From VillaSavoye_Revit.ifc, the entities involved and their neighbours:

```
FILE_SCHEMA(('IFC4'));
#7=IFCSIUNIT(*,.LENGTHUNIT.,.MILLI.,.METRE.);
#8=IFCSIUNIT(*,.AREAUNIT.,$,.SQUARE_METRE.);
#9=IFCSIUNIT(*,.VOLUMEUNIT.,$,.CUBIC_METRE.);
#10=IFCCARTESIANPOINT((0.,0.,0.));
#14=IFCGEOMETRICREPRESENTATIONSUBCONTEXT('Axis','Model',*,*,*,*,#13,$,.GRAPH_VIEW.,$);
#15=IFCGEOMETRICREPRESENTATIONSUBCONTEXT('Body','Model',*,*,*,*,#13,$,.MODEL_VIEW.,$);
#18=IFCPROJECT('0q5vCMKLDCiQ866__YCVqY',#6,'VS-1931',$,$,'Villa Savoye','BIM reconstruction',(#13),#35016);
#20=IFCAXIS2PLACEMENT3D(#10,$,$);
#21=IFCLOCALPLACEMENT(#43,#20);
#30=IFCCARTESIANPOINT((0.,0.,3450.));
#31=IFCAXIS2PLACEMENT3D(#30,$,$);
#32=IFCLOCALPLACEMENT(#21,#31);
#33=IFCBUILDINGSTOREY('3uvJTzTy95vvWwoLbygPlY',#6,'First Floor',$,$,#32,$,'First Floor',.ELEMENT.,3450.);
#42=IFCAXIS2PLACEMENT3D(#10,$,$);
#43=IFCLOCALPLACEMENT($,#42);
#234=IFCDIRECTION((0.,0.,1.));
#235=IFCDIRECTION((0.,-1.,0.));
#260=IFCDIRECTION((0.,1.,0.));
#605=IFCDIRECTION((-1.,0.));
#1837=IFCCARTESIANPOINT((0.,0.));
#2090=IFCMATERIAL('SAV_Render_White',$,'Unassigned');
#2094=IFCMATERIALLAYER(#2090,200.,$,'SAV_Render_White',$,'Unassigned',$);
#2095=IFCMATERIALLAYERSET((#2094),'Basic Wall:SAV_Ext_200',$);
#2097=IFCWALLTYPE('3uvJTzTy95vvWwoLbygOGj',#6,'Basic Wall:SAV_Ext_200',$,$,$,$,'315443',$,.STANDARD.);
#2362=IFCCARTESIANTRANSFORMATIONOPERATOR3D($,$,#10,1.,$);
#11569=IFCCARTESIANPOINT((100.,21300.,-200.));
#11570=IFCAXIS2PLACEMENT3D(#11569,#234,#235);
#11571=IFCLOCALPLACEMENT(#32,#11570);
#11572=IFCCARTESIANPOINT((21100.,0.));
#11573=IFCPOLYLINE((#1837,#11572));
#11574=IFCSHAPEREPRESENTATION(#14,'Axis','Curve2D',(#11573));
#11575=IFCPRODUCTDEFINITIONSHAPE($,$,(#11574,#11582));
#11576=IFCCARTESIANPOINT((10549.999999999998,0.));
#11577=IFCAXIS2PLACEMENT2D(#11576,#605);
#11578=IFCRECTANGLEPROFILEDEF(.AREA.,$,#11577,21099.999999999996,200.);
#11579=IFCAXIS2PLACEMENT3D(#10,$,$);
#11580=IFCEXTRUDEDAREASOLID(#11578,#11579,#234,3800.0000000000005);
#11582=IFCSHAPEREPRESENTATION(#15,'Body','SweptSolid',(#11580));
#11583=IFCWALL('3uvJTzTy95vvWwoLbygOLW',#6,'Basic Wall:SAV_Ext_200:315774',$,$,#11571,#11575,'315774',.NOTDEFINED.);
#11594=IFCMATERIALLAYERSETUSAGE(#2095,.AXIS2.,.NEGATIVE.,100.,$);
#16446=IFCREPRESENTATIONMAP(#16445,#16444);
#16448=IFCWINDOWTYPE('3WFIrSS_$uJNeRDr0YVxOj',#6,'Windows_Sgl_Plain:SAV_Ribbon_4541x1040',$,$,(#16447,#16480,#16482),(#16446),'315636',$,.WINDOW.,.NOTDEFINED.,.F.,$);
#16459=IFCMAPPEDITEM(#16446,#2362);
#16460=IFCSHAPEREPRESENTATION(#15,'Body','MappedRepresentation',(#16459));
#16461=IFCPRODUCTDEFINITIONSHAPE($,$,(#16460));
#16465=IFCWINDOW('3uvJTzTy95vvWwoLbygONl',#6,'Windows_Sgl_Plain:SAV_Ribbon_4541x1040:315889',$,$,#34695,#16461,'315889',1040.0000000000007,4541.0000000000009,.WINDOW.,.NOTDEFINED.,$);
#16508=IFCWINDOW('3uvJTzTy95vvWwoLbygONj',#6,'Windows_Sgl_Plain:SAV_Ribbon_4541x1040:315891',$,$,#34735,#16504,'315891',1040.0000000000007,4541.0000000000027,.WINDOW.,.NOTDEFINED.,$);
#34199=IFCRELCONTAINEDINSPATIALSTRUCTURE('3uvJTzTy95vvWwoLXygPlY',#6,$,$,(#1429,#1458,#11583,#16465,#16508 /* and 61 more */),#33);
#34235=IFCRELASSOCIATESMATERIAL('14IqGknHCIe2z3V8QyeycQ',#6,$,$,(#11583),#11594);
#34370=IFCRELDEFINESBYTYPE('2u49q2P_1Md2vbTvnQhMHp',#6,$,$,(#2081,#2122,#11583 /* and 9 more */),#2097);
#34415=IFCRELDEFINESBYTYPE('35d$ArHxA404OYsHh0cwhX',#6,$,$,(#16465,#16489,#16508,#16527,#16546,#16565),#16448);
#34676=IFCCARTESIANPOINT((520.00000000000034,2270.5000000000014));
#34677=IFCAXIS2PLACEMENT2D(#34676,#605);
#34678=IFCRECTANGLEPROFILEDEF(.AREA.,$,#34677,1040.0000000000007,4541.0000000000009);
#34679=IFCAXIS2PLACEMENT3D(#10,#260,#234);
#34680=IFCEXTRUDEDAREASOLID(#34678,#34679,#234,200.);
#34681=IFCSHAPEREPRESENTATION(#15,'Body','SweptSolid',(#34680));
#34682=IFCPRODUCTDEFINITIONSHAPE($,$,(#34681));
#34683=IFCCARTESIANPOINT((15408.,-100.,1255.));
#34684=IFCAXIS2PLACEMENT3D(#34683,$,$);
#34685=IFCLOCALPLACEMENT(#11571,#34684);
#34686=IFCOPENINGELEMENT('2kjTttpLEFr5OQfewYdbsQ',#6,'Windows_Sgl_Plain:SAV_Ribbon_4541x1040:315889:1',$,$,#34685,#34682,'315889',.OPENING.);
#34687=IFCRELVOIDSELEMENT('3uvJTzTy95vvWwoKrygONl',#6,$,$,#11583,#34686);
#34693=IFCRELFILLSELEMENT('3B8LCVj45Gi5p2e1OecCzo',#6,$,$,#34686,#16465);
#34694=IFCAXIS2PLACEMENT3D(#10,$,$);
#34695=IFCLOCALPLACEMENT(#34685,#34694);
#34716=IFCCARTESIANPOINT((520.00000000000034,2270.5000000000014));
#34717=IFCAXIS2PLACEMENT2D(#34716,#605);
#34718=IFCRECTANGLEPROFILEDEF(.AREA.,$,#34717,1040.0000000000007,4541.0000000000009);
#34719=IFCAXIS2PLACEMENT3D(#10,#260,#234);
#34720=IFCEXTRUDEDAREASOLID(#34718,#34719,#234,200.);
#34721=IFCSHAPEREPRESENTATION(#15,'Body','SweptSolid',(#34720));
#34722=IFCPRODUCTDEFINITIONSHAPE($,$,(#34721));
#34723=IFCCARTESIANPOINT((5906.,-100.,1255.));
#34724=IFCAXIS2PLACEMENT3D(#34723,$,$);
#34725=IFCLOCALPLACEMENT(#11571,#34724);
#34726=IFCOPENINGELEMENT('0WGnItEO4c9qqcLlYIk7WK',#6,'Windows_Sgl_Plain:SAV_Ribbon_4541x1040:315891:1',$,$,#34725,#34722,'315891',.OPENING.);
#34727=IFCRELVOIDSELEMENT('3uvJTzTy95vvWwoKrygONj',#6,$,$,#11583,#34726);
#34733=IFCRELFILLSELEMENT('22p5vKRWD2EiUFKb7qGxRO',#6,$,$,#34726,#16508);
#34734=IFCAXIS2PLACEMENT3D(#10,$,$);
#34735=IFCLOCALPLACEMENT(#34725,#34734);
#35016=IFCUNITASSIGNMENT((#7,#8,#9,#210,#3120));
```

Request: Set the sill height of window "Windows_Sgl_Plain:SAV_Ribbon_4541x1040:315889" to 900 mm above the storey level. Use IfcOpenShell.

```python
import numpy as np
import ifcopenshell
import ifcopenshell.api.geometry
import ifcopenshell.geom
import ifcopenshell.util.element
import ifcopenshell.util.placement
import ifcopenshell.util.shape
import ifcopenshell.util.unit

model = ifcopenshell.open("VillaSavoye_Revit.ifc")
unit_scale = ifcopenshell.util.unit.calculate_unit_scale(model)

window = model.by_guid("3uvJTzTy95vvWwoLbygONl")
opening = window.FillsVoids[0].RelatingOpeningElement
storey = ifcopenshell.util.element.get_container(window, ifc_class="IfcBuildingStorey")
level = ifcopenshell.util.placement.get_local_placement(storey.ObjectPlacement)[2, 3]

# The opening's origin need not be at the sill, so measure its lowest point.
shape = ifcopenshell.geom.create_shape(ifcopenshell.geom.settings(), opening)
bottom = ifcopenshell.util.shape.get_shape_bottom_elevation(shape, shape.geometry) / unit_scale
dz = level + 900.0 - bottom

shift = np.array([0.0, 0.0, dz])
# The window is placed relative to its opening, so it follows when the opening moves.
matrix = ifcopenshell.util.placement.get_local_placement(opening.ObjectPlacement)
matrix[:3, 3] += shift
ifcopenshell.api.geometry.edit_object_placement(
    model, product=opening, matrix=matrix, is_si=False, should_transform_children=True
)

print(f"moved by {dz * unit_scale:+.3f} m")

model.write("VillaSavoye_Revit-out.ifc")
```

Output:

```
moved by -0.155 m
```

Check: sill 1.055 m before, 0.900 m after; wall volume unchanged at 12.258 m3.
